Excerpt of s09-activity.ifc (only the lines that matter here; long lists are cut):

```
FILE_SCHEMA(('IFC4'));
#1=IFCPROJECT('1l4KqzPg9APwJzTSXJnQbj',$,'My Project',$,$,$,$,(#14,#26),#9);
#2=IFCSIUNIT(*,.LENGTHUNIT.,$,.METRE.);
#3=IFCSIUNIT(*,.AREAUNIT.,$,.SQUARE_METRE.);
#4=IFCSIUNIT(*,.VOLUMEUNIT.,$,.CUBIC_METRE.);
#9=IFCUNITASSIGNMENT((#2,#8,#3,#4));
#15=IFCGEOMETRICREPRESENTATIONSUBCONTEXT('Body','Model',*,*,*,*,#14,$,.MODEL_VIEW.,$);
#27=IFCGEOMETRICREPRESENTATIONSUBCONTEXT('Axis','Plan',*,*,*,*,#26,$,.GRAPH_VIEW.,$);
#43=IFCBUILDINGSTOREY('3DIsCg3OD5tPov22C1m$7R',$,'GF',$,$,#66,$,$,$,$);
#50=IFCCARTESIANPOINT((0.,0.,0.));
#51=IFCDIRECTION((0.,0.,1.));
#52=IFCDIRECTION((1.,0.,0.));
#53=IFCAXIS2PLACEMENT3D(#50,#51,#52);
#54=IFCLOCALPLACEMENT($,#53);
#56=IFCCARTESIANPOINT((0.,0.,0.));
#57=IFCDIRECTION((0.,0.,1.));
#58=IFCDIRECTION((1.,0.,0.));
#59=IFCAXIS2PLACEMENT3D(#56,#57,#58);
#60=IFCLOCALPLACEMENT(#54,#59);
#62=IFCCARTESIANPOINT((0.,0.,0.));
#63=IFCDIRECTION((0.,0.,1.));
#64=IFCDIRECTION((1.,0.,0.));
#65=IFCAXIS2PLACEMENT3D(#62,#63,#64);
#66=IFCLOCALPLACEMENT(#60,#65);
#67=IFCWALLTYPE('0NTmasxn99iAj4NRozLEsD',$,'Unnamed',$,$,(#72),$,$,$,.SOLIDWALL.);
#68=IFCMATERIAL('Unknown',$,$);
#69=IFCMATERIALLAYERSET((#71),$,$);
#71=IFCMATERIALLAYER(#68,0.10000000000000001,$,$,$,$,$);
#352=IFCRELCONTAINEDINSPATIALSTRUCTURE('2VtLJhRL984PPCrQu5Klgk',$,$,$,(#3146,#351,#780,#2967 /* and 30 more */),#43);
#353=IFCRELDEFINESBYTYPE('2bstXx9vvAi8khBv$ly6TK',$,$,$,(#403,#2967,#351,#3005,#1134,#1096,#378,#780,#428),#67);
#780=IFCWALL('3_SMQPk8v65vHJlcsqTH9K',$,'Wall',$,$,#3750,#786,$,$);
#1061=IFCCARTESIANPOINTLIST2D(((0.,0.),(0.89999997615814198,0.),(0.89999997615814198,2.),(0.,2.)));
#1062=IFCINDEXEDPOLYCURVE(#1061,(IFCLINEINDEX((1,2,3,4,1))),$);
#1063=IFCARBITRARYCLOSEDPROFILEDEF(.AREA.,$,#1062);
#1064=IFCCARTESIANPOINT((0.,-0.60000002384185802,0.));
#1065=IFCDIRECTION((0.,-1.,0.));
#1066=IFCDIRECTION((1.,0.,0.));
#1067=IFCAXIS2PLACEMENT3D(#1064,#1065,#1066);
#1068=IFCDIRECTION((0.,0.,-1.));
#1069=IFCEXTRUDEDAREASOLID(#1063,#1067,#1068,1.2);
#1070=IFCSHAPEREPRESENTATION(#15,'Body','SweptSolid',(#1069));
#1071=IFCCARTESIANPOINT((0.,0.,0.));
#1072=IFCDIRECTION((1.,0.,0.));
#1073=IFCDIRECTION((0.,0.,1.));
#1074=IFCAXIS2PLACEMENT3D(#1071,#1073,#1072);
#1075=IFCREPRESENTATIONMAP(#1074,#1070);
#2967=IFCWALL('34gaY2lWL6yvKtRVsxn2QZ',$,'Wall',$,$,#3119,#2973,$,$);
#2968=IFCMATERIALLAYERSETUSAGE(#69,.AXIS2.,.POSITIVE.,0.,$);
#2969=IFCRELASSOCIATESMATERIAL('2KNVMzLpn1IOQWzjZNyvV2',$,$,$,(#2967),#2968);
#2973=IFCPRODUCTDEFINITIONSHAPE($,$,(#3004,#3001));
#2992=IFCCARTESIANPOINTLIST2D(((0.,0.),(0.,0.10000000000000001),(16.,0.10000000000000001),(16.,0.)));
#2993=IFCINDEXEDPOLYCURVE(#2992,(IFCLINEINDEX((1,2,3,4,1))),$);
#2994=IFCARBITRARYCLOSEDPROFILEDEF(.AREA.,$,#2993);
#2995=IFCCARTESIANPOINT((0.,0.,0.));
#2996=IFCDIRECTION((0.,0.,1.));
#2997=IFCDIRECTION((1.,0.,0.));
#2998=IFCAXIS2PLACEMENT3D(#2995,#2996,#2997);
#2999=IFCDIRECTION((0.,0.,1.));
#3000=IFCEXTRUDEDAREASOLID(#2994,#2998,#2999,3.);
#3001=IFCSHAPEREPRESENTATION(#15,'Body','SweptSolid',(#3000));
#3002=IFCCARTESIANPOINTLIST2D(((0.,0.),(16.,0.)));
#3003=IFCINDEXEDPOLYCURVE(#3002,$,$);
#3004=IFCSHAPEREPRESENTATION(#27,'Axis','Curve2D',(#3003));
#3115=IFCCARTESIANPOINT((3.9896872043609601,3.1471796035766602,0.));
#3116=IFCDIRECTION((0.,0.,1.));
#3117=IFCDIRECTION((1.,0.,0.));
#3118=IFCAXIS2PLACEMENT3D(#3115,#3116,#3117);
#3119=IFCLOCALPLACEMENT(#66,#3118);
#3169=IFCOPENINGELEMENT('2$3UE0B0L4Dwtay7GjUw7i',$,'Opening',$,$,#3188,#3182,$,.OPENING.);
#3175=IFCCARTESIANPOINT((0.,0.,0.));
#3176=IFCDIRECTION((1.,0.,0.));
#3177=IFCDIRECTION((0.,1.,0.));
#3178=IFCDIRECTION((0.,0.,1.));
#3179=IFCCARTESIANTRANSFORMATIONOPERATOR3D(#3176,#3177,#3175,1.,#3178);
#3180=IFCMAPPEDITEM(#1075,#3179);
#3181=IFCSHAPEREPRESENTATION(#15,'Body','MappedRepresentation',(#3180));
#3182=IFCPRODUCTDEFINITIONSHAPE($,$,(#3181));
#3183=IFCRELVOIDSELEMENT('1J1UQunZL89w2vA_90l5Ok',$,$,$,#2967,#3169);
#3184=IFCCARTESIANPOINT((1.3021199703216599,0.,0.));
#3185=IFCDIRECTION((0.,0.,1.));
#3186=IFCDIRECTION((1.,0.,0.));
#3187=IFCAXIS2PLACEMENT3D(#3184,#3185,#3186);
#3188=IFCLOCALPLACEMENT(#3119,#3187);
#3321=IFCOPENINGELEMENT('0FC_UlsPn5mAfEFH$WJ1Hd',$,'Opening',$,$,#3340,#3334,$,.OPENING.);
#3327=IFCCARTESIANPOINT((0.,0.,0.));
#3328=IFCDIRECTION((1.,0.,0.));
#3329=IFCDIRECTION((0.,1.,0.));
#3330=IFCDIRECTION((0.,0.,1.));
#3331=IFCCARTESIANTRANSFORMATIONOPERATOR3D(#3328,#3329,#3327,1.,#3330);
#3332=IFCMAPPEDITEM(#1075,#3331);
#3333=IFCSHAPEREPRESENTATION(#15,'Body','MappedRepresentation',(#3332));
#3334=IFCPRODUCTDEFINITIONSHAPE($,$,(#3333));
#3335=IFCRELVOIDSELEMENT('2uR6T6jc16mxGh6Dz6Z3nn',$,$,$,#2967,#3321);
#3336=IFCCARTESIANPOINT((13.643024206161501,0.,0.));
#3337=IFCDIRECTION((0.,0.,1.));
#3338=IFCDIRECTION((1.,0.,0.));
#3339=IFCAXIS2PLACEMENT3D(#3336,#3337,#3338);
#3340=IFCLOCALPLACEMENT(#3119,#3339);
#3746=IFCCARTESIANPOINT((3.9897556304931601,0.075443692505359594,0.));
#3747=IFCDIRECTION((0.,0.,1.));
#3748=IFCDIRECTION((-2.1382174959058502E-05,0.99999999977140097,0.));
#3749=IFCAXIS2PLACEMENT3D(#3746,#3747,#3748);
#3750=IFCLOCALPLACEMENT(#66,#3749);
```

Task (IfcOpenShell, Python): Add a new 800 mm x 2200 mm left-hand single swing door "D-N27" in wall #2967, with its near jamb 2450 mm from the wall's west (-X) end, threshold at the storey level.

```python
import numpy as np
import ifcopenshell
import ifcopenshell.api.feature
import ifcopenshell.api.geometry
import ifcopenshell.api.root
import ifcopenshell.api.spatial
import ifcopenshell.geom
import ifcopenshell.util.element
import ifcopenshell.util.placement
import ifcopenshell.util.representation
import ifcopenshell.util.shape
import ifcopenshell.util.unit

model = ifcopenshell.open("s09-activity.ifc")
unit_scale = ifcopenshell.util.unit.calculate_unit_scale(model)
settings = ifcopenshell.geom.settings()


def volume(element):
    """Net volume in cubic metres, openings subtracted."""
    shape = ifcopenshell.geom.create_shape(settings, element)
    return ifcopenshell.util.shape.get_volume(shape.geometry)


wall = model.by_guid("34gaY2lWL6yvKtRVsxn2QZ")
storey = ifcopenshell.util.element.get_container(wall, ifc_class="IfcBuildingStorey")
context = ifcopenshell.util.representation.get_context(model, "Model", "Body", "MODEL_VIEW")
before = volume(wall)

width, height, from_end, sill = 0.8, 2.2, 2.45, 0.0  # metres

# The wall runs along its own X axis, and the end named is its -X end.
wall_shape = ifcopenshell.geom.create_shape(settings, wall)
x, y, z = ifcopenshell.util.shape.get_vertices(wall_shape.geometry).T
start = x.min() + from_end
face, thickness = float(y.min()), float(y.max() - y.min())
wall_matrix = ifcopenshell.util.placement.get_local_placement(wall.ObjectPlacement)
level = ifcopenshell.util.placement.get_local_placement(storey.ObjectPlacement)[2, 3]


def in_wall(x, y):
    """Placement at x, y metres in the wall's axes, at sill height."""
    matrix = wall_matrix.copy()
    matrix[:, 3] = wall_matrix @ np.array([x / unit_scale, y / unit_scale, 0.0, 1.0])
    matrix[2, 3] = level + sill / unit_scale
    return matrix


# Opening: a box that overshoots both wall faces by 50 mm.
opening = ifcopenshell.api.root.create_entity(model, ifc_class="IfcOpeningElement", predefined_type="OPENING")
box = ifcopenshell.api.geometry.add_wall_representation(
    model, context=context, length=width, height=height, thickness=thickness + 0.1
)
ifcopenshell.api.geometry.assign_representation(model, product=opening, representation=box)
ifcopenshell.api.geometry.edit_object_placement(model, product=opening, matrix=in_wall(start, face - 0.05), is_si=False)
ifcopenshell.api.feature.add_feature(model, feature=opening, element=wall)

door = ifcopenshell.api.root.create_entity(model, ifc_class="IfcDoor", name="D-N27", predefined_type="DOOR")
door.OverallWidth, door.OverallHeight = width / unit_scale, height / unit_scale
door.OperationType = "SINGLE_SWING_LEFT"
body = ifcopenshell.api.geometry.add_door_representation(
    model,
    context=context,
    overall_width=door.OverallWidth,
    overall_height=door.OverallHeight,
    operation_type="SINGLE_SWING_LEFT",
    lining_properties={"LiningDepth": thickness / unit_scale, "ThresholdDepth": thickness / unit_scale},
)
ifcopenshell.api.geometry.assign_representation(model, product=door, representation=body)
ifcopenshell.api.spatial.assign_container(model, products=[door], relating_structure=storey)
ifcopenshell.api.feature.add_filling(model, opening=opening, element=door)

# The lining spans the wall, so the door starts at the wall face.
ifcopenshell.api.geometry.edit_object_placement(model, product=door, matrix=in_wall(start, face), is_si=False)

after = volume(wall)

print(f"wall volume {before:.3f} -> {after:.3f} m3")

model.write("s09-activity_rev.ifc")
```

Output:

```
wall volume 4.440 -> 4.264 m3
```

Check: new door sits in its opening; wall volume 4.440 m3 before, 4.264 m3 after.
